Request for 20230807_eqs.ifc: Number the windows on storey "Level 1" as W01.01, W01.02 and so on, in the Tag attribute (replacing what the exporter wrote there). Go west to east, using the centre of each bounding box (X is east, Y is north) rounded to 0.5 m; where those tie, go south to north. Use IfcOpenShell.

First a look at what the model holds.

```python
import ifcopenshell
import ifcopenshell.util.element
import ifcopenshell.util.placement

model = ifcopenshell.open("20230807_eqs.ifc")
print(model.schema)
storey = next(s for s in model.by_type("IfcBuildingStorey") if s.Name == "Level 1")
windows = [e for e in ifcopenshell.util.element.get_decomposition(storey) if e.is_a("IfcWindow")]
for e in sorted(windows, key=lambda e: e.id()):
    origin = ifcopenshell.util.placement.get_local_placement(e.ObjectPlacement)[:3, 3]
    print(e.id(), e.Tag, e.Name, origin.round(2) + 0.0, sep=" | ")
```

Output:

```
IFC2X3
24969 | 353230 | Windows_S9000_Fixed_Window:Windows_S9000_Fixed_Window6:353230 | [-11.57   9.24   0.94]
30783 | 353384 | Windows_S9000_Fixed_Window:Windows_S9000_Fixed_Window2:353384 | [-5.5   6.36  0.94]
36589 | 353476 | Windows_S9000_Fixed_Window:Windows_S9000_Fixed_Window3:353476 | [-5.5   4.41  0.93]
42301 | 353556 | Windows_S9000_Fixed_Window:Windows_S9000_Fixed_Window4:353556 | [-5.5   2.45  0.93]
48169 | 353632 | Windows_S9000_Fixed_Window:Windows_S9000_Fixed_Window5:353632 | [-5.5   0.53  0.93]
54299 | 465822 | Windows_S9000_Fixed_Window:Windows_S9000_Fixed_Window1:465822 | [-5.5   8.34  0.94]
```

```python
import ifcopenshell
import ifcopenshell.geom
import ifcopenshell.util.element
import ifcopenshell.util.shape

model = ifcopenshell.open("20230807_eqs.ifc")
settings = ifcopenshell.geom.settings()
settings.set("use-world-coords", True)


def centre(element):
    shape = ifcopenshell.geom.create_shape(settings, element)
    return ifcopenshell.util.shape.get_bbox_centroid(shape.geometry)


storey = next(s for s in model.by_type("IfcBuildingStorey") if s.Name == "Level 1")
windows = [e for e in ifcopenshell.util.element.get_decomposition(storey) if e.is_a("IfcWindow")]

# Insertion points can sit at a corner or the storey origin, so sort by the geometry (in metres).
centres = {e: centre(e) for e in windows}
windows.sort(key=lambda e: (round(centres[e][0] / 0.5), centres[e][1]))

for i, e in enumerate(windows, start=1):
    number = f"W01.{i:02d}"
    e.Tag = number
    print(e.id(), number)

model.write("20230807_eqs_v2.ifc")
```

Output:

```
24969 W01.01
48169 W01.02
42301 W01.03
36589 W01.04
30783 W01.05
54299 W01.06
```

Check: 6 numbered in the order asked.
